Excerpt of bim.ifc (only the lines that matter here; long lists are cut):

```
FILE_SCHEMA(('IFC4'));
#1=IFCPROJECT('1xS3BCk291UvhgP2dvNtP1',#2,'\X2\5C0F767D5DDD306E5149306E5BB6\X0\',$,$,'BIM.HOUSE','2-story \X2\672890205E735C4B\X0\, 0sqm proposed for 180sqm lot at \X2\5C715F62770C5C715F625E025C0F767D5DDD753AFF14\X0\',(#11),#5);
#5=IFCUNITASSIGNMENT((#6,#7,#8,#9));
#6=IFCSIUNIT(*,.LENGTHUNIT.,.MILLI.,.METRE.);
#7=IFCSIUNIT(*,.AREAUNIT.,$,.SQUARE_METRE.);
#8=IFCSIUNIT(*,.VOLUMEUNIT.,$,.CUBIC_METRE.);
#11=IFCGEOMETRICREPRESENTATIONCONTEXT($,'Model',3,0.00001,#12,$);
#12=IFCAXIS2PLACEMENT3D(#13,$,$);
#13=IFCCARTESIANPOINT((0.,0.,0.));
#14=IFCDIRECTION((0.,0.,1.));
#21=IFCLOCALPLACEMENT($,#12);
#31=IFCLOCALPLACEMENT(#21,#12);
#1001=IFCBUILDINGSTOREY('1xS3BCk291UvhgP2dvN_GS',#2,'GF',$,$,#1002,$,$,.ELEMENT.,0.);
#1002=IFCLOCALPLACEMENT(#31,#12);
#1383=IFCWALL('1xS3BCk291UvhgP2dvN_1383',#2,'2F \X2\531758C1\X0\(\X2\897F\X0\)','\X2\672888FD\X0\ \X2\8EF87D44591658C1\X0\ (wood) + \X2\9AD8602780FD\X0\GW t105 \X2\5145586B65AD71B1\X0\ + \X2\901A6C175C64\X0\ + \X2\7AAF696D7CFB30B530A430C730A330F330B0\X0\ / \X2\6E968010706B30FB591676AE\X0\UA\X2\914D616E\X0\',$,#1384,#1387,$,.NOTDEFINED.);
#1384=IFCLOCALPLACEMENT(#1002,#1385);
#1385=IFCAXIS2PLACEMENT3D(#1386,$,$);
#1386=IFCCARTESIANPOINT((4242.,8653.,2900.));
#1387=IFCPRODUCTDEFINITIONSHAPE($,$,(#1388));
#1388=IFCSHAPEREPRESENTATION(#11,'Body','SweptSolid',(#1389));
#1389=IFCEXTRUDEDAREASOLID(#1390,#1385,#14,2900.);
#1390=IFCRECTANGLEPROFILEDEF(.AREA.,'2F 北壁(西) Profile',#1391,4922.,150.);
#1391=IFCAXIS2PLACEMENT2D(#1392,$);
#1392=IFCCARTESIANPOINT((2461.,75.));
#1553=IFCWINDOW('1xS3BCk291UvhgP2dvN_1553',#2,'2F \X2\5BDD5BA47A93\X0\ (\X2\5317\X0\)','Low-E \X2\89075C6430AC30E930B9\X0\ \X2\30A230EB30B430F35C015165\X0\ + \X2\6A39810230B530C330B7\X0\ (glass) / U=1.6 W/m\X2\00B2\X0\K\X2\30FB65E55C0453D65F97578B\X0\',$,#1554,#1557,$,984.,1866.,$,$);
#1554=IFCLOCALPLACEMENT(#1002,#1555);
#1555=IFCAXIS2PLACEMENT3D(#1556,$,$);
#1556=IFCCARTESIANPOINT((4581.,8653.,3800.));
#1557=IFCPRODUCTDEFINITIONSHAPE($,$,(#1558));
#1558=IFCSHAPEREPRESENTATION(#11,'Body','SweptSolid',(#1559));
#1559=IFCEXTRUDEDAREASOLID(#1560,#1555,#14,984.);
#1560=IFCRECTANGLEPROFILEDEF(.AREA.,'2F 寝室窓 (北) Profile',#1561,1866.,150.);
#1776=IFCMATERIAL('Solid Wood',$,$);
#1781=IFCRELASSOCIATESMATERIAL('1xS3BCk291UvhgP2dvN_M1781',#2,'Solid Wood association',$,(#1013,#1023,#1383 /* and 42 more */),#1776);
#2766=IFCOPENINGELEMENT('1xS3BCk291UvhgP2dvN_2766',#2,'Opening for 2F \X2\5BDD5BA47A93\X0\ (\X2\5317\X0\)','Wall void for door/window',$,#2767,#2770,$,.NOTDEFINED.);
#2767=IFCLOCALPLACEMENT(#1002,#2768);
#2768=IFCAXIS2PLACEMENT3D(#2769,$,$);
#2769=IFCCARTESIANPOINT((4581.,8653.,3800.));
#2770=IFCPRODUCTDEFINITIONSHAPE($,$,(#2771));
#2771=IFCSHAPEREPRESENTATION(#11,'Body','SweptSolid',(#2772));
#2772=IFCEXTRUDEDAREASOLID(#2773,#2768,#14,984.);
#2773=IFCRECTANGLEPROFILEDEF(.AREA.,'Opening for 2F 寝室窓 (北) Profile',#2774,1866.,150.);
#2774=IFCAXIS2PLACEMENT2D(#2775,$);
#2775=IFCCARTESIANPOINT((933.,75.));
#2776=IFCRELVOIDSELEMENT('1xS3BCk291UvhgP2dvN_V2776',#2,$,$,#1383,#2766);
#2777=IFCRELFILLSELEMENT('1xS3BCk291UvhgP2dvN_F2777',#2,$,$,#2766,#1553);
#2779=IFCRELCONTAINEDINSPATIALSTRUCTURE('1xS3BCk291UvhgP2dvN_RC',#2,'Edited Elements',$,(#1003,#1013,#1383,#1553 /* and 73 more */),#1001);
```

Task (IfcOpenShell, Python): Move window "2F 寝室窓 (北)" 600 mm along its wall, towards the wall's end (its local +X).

```python
import ifcopenshell
import ifcopenshell.api.geometry
import ifcopenshell.util.placement
import ifcopenshell.util.unit

model = ifcopenshell.open("bim.ifc")
unit_scale = ifcopenshell.util.unit.calculate_unit_scale(model)

window = model.by_id(1553)
opening = window.FillsVoids[0].RelatingOpeningElement
wall = opening.VoidsElements[0].RelatingBuildingElement

wall_matrix = ifcopenshell.util.placement.get_local_placement(wall.ObjectPlacement)
shift = wall_matrix[:3, 0] * 0.6 / unit_scale
before = ifcopenshell.util.placement.get_local_placement(window.ObjectPlacement)[:3, 3].copy()

# The window is not placed relative to its opening, so move both.
for product in (opening, window):
    matrix = ifcopenshell.util.placement.get_local_placement(product.ObjectPlacement)
    matrix[:3, 3] += shift
    ifcopenshell.api.geometry.edit_object_placement(model, product=product, matrix=matrix, is_si=False)

after = ifcopenshell.util.placement.get_local_placement(window.ObjectPlacement)[:3, 3]
print("window moved by", (after - before).round(3) + 0.0)

model.write("bim-out.ifc")
```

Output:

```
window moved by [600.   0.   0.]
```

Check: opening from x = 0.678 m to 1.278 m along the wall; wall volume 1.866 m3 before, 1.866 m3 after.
